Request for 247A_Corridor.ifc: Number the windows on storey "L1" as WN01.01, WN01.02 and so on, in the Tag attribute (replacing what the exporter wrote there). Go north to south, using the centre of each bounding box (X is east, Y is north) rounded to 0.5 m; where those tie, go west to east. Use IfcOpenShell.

First a look at what the model holds.

```python
import ifcopenshell
import ifcopenshell.util.element
import ifcopenshell.util.placement

model = ifcopenshell.open("247A_Corridor.ifc")
print(model.schema)
storey = next(s for s in model.by_type("IfcBuildingStorey") if s.Name == "L1")
windows = [e for e in ifcopenshell.util.element.get_decomposition(storey) if e.is_a("IfcWindow")]
for e in sorted(windows, key=lambda e: e.id()):
    origin = ifcopenshell.util.placement.get_local_placement(e.ObjectPlacement)[:3, 3]
    print(e.id(), e.Tag, e.Name, origin.round(2) + 0.0, sep=" | ")
```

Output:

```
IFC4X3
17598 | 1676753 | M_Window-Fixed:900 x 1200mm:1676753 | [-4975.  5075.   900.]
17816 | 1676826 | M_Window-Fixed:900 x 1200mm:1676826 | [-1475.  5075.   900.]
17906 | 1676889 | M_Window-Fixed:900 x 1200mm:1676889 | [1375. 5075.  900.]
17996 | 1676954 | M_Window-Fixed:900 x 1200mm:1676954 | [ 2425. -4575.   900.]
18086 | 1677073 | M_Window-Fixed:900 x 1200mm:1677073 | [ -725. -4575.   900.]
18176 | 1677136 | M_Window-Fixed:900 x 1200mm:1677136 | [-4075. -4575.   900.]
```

```python
import ifcopenshell
import ifcopenshell.geom
import ifcopenshell.util.element
import ifcopenshell.util.shape

model = ifcopenshell.open("247A_Corridor.ifc")
settings = ifcopenshell.geom.settings()
settings.set("use-world-coords", True)


def centre(element):
    shape = ifcopenshell.geom.create_shape(settings, element)
    return ifcopenshell.util.shape.get_bbox_centroid(shape.geometry)


storey = next(s for s in model.by_type("IfcBuildingStorey") if s.Name == "L1")
windows = [e for e in ifcopenshell.util.element.get_decomposition(storey) if e.is_a("IfcWindow")]

# Insertion points can sit at a corner or the storey origin, so sort by the geometry (in metres).
centres = {e: centre(e) for e in windows}
windows.sort(key=lambda e: (-round(centres[e][1] / 0.5), centres[e][0]))

for i, e in enumerate(windows, start=1):
    number = f"WN01.{i:02d}"
    e.Tag = number
    print(e.id(), number)

model.write("247A_Corridor_rev.ifc")
```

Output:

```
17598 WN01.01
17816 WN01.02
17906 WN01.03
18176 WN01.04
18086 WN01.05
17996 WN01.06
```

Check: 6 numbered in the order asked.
